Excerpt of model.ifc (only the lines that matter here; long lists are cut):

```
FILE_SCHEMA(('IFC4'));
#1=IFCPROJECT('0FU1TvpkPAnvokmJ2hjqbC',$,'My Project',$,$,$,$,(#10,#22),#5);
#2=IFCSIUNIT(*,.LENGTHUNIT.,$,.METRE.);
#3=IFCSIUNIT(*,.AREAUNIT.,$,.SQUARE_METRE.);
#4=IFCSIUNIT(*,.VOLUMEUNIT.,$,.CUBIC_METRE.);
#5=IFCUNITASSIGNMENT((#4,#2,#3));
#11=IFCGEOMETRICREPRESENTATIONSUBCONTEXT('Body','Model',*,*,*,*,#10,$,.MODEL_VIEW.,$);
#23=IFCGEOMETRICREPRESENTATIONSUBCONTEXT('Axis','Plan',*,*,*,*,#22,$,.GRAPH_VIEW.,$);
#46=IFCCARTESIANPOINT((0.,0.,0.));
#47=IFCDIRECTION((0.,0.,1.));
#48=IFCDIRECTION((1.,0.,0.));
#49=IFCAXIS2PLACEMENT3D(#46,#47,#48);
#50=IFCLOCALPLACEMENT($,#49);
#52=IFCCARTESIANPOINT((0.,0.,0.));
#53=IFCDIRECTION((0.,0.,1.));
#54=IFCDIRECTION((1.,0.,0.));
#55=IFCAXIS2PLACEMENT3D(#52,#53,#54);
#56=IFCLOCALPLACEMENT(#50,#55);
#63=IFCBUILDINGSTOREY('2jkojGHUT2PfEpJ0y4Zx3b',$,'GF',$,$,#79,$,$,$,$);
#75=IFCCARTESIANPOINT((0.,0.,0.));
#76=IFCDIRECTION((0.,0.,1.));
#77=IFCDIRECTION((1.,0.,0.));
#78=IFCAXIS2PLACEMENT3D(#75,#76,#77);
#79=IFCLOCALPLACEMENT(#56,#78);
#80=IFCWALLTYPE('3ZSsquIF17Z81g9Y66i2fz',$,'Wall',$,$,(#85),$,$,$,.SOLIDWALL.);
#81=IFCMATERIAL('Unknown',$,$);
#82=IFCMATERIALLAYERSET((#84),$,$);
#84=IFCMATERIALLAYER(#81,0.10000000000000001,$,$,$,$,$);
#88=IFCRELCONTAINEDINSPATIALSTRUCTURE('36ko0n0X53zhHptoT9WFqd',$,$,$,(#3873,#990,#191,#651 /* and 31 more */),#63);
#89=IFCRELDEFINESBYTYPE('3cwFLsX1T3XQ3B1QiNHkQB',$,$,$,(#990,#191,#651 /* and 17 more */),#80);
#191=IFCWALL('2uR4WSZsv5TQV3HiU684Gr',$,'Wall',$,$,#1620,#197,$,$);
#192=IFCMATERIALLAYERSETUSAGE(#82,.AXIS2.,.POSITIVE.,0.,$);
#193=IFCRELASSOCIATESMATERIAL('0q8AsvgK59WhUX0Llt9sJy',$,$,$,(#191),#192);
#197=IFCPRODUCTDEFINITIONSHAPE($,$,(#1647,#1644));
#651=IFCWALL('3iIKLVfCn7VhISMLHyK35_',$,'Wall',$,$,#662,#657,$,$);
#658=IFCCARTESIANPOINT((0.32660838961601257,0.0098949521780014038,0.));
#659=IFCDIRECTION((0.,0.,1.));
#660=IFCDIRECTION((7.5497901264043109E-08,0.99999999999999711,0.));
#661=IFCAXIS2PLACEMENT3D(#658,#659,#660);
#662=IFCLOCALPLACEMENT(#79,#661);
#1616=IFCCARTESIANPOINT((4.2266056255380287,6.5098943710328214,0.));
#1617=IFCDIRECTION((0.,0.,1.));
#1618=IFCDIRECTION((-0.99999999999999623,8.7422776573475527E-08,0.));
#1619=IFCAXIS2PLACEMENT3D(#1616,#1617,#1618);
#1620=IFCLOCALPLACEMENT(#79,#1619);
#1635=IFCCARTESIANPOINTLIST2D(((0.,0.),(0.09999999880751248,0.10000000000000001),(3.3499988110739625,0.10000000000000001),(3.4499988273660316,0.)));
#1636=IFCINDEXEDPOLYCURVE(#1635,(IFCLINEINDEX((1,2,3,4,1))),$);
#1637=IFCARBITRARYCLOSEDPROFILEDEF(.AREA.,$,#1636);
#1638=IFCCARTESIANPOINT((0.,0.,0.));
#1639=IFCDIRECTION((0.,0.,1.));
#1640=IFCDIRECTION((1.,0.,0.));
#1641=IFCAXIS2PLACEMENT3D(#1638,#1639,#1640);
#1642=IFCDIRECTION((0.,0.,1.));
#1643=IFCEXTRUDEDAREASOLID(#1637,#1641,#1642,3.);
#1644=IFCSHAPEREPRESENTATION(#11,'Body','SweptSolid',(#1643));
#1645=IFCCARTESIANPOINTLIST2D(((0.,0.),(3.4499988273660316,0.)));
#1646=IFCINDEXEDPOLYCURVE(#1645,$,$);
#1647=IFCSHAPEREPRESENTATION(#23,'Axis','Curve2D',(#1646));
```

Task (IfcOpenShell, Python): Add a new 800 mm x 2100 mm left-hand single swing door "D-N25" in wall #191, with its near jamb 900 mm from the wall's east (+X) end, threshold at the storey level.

```python
import numpy as np
import ifcopenshell
import ifcopenshell.api.feature
import ifcopenshell.api.geometry
import ifcopenshell.api.root
import ifcopenshell.api.spatial
import ifcopenshell.geom
import ifcopenshell.util.element
import ifcopenshell.util.placement
import ifcopenshell.util.representation
import ifcopenshell.util.shape
import ifcopenshell.util.unit

model = ifcopenshell.open("model.ifc")
unit_scale = ifcopenshell.util.unit.calculate_unit_scale(model)
settings = ifcopenshell.geom.settings()


def volume(element):
    """Net volume in cubic metres, openings subtracted."""
    shape = ifcopenshell.geom.create_shape(settings, element)
    return ifcopenshell.util.shape.get_volume(shape.geometry)


wall = model.by_guid("2uR4WSZsv5TQV3HiU684Gr")
storey = ifcopenshell.util.element.get_container(wall, ifc_class="IfcBuildingStorey")
context = ifcopenshell.util.representation.get_context(model, "Model", "Body", "MODEL_VIEW")
before = volume(wall)

width, height, from_end, sill = 0.8, 2.1, 0.9, 0.0  # metres

# The wall runs along its own X axis, and the end named is its -X end.
wall_shape = ifcopenshell.geom.create_shape(settings, wall)
x, y, z = ifcopenshell.util.shape.get_vertices(wall_shape.geometry).T
start = x.min() + from_end
face, thickness = float(y.min()), float(y.max() - y.min())
wall_matrix = ifcopenshell.util.placement.get_local_placement(wall.ObjectPlacement)
level = ifcopenshell.util.placement.get_local_placement(storey.ObjectPlacement)[2, 3]


def in_wall(x, y):
    """Placement at x, y metres in the wall's axes, at sill height."""
    matrix = wall_matrix.copy()
    matrix[:, 3] = wall_matrix @ np.array([x / unit_scale, y / unit_scale, 0.0, 1.0])
    matrix[2, 3] = level + sill / unit_scale
    return matrix


# Opening: a box that overshoots both wall faces by 50 mm.
opening = ifcopenshell.api.root.create_entity(model, ifc_class="IfcOpeningElement", predefined_type="OPENING")
box = ifcopenshell.api.geometry.add_wall_representation(
    model, context=context, length=width, height=height, thickness=thickness + 0.1
)
ifcopenshell.api.geometry.assign_representation(model, product=opening, representation=box)
ifcopenshell.api.geometry.edit_object_placement(model, product=opening, matrix=in_wall(start, face - 0.05), is_si=False)
ifcopenshell.api.feature.add_feature(model, feature=opening, element=wall)

door = ifcopenshell.api.root.create_entity(model, ifc_class="IfcDoor", name="D-N25", predefined_type="DOOR")
door.OverallWidth, door.OverallHeight = width / unit_scale, height / unit_scale
door.OperationType = "SINGLE_SWING_LEFT"
body = ifcopenshell.api.geometry.add_door_representation(
    model,
    context=context,
    overall_width=door.OverallWidth,
    overall_height=door.OverallHeight,
    operation_type="SINGLE_SWING_LEFT",
    lining_properties={"LiningDepth": thickness / unit_scale, "ThresholdDepth": thickness / unit_scale},
)
ifcopenshell.api.geometry.assign_representation(model, product=door, representation=body)
ifcopenshell.api.spatial.assign_container(model, products=[door], relating_structure=storey)
ifcopenshell.api.feature.add_filling(model, opening=opening, element=door)

# The lining spans the wall, so the door starts at the wall face.
ifcopenshell.api.geometry.edit_object_placement(model, product=door, matrix=in_wall(start, face), is_si=False)

after = volume(wall)

print(f"wall volume {before:.3f} -> {after:.3f} m3")

model.write("model-out.ifc")
```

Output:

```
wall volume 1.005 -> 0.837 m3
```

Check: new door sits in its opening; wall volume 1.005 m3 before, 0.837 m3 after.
